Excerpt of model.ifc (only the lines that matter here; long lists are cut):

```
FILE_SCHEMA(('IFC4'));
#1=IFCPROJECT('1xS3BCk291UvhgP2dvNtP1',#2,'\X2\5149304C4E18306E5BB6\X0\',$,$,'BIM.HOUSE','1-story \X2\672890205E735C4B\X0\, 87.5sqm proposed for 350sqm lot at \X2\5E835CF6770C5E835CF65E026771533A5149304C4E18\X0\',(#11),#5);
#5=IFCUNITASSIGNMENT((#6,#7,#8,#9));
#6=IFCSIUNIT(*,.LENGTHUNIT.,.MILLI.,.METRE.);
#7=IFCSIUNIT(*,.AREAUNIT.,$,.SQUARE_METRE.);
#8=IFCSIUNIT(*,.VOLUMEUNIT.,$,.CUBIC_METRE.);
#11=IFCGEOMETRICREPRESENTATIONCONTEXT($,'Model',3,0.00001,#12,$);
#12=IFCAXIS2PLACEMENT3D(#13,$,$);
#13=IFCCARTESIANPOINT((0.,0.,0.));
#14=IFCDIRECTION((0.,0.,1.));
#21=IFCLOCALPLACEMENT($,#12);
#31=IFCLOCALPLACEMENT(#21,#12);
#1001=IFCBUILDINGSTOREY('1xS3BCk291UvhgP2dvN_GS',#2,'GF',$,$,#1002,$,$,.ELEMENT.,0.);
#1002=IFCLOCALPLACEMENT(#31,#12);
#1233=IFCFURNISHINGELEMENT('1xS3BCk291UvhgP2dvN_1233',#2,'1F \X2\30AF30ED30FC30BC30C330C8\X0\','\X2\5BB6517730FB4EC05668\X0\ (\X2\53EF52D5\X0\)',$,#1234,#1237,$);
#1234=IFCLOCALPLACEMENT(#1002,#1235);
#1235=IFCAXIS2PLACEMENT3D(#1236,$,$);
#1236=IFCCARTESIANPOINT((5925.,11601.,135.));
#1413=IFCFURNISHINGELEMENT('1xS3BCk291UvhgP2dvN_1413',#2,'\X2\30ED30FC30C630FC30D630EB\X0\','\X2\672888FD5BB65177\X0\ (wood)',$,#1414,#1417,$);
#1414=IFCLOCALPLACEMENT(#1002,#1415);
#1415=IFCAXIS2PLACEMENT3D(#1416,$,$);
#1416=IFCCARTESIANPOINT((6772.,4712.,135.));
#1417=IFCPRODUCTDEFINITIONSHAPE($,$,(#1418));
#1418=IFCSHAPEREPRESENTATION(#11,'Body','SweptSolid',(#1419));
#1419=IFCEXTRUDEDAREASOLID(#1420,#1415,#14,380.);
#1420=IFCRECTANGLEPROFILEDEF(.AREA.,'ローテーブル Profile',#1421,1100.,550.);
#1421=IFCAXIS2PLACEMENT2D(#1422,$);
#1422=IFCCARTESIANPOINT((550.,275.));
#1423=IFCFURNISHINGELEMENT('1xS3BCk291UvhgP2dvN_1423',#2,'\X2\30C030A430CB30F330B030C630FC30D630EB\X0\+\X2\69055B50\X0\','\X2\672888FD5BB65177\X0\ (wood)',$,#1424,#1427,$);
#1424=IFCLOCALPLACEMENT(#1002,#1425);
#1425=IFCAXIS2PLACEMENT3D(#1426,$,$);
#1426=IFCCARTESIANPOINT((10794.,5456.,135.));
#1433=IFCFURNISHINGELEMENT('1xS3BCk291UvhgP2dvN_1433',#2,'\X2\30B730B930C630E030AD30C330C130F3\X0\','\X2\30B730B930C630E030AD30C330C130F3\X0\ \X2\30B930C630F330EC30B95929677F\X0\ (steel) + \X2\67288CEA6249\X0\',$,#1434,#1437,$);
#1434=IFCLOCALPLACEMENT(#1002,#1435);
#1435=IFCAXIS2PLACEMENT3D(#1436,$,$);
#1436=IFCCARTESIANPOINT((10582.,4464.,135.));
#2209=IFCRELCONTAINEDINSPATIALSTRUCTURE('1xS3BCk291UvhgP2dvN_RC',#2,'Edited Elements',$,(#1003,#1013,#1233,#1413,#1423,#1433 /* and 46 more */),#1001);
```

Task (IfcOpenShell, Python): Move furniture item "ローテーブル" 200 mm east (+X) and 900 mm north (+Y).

```python
import ifcopenshell
import ifcopenshell.api.geometry
import ifcopenshell.util.placement

model = ifcopenshell.open("model.ifc")

item = model.by_guid("1xS3BCk291UvhgP2dvN_1413")
matrix = ifcopenshell.util.placement.get_local_placement(item.ObjectPlacement)
matrix[0, 3] += 200.0
matrix[1, 3] += 900.0
ifcopenshell.api.geometry.edit_object_placement(model, product=item, matrix=matrix, is_si=False)

print(ifcopenshell.util.placement.get_local_placement(item.ObjectPlacement).round(3) + 0.0)

model.write("model_v2.ifc")
```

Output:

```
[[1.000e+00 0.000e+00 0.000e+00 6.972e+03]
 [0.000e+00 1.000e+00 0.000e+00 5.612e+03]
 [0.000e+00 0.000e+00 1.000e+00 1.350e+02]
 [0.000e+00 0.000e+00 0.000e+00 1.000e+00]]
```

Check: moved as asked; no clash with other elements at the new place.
